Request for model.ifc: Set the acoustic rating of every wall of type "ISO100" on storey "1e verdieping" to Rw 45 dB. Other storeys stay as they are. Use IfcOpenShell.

First a look at what the model holds.

```python
import ifcopenshell
import ifcopenshell.util.element

model = ifcopenshell.open("model.ifc")
print(model.schema)
storey = next(s for s in model.by_type("IfcBuildingStorey") if s.Name == "1e verdieping")
walls = [e for e in ifcopenshell.util.element.get_decomposition(storey) if e.is_a("IfcWall")]
seen = {}
for e in walls:
    element_type = ifcopenshell.util.element.get_type(e)
    key = (element_type.Name if element_type != e and element_type else None, ifcopenshell.util.element.get_pset(e, "Pset_WallCommon", "AcousticRating"))
    seen[key] = seen.get(key, 0) + 1
for (name, value), count in sorted(seen.items(), key=str):
    print(count, "x", name, "|", value)
```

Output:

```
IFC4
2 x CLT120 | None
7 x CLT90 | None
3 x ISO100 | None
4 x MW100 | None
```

```python
import ifcopenshell
import ifcopenshell.api.pset
import ifcopenshell.util.element

model = ifcopenshell.open("model.ifc")

storey = next(s for s in model.by_type("IfcBuildingStorey") if s.Name == "1e verdieping")
walls = [e for e in ifcopenshell.util.element.get_decomposition(storey) if e.is_a("IfcWall")]

count = 0
for e in walls:
    element_type = ifcopenshell.util.element.get_type(e)
    if element_type in (None, e) or element_type.Name != "ISO100":
        continue
    # add_pset returns the element's existing set when there is one.
    pset = ifcopenshell.api.pset.add_pset(model, product=e, name="Pset_WallCommon")
    ifcopenshell.api.pset.edit_pset(model, pset=pset, properties={"AcousticRating": "Rw 45 dB"})
    count += 1

print(count, "walls updated")

model.write("model_rev.ifc")
```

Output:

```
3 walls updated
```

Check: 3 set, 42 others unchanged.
